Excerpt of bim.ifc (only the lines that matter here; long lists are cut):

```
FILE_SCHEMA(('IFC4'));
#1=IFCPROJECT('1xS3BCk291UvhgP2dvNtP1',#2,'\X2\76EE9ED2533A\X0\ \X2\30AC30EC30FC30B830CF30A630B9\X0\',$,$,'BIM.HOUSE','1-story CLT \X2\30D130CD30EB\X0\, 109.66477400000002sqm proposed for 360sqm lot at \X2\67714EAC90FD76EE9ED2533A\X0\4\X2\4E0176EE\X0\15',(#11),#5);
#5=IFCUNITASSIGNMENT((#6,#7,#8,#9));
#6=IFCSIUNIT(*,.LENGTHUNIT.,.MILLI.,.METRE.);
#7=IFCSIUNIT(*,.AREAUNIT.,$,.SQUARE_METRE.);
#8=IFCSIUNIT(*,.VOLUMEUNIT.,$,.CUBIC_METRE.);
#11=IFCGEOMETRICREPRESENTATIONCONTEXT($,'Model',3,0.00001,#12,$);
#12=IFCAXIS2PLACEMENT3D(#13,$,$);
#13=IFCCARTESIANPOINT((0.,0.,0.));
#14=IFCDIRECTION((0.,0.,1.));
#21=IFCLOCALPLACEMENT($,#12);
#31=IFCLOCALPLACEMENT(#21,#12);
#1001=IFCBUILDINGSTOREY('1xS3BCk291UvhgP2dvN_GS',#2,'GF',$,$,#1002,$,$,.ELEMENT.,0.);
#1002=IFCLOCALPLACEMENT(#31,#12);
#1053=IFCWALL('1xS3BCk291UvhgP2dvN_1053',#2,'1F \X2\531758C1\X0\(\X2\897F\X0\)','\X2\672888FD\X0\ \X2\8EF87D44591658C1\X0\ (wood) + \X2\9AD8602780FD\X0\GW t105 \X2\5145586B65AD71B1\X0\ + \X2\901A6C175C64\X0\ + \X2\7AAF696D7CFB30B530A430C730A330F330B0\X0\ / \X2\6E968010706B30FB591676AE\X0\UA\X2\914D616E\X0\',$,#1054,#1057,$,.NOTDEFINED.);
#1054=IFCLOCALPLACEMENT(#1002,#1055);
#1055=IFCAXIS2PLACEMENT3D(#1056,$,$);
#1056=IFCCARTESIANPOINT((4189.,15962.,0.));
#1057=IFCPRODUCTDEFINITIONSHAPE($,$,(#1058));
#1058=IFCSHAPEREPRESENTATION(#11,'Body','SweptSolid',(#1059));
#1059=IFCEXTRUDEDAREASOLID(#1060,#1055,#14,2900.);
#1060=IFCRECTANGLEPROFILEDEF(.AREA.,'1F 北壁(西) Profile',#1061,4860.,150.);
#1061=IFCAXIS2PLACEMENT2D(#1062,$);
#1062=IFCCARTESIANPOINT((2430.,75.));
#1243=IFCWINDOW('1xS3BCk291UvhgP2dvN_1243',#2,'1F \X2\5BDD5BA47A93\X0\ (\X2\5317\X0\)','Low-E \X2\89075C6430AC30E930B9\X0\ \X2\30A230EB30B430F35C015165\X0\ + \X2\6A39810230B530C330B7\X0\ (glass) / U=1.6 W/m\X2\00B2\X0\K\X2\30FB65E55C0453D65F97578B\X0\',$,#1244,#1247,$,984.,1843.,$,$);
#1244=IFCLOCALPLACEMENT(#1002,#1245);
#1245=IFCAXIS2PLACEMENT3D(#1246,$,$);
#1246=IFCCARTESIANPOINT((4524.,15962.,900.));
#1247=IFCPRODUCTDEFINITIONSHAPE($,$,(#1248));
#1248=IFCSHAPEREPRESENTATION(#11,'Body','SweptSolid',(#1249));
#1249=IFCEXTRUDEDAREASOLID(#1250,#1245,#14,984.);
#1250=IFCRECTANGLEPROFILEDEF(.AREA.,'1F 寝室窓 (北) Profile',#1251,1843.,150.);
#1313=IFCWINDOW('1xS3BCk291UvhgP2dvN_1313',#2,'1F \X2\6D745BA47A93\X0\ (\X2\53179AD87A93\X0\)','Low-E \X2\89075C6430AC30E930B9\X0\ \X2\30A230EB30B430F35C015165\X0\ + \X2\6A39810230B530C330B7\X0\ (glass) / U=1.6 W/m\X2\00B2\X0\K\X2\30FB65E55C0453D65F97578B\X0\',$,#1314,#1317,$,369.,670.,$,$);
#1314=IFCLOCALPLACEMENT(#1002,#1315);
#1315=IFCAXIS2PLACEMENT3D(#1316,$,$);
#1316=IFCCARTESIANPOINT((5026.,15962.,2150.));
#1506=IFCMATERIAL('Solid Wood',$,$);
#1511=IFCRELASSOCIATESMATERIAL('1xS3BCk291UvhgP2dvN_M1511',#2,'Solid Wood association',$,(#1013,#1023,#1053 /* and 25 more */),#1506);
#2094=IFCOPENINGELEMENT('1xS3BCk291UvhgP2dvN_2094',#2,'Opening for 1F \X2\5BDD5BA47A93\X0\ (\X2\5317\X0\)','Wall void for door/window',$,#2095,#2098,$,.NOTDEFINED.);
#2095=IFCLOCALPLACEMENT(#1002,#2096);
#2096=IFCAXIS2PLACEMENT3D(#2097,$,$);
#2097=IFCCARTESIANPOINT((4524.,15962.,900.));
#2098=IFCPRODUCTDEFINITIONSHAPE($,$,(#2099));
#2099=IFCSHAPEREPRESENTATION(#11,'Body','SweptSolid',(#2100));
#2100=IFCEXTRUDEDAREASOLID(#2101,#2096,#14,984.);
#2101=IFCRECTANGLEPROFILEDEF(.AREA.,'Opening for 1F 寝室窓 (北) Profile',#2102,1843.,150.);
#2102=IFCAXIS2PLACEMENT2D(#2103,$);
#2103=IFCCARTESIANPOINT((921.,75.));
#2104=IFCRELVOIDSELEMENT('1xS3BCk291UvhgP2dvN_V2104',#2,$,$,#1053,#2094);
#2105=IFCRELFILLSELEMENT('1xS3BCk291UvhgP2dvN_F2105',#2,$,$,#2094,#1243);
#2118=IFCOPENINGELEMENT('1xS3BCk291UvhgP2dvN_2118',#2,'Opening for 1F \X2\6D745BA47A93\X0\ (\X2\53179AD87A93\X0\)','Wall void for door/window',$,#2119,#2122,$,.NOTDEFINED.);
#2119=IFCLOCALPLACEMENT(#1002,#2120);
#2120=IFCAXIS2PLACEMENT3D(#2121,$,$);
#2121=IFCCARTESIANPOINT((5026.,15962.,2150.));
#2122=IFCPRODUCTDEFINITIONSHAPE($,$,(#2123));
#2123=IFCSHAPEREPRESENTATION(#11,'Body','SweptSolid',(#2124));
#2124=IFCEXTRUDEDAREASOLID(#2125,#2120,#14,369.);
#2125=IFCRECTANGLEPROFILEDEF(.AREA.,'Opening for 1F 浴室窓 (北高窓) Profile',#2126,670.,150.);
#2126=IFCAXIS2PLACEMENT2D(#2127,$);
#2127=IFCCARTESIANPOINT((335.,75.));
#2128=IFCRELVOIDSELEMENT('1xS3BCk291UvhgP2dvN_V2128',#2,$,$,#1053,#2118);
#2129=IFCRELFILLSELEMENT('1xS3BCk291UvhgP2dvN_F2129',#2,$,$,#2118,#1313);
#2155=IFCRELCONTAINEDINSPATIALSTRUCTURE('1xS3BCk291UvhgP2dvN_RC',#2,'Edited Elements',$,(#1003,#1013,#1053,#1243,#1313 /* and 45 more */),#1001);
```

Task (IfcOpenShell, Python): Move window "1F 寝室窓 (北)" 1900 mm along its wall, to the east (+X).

```python
import ifcopenshell
import ifcopenshell.api.geometry
import ifcopenshell.util.placement
import ifcopenshell.util.unit

model = ifcopenshell.open("bim.ifc")
unit_scale = ifcopenshell.util.unit.calculate_unit_scale(model)

window = model.by_guid("1xS3BCk291UvhgP2dvN_1243")
opening = window.FillsVoids[0].RelatingOpeningElement
wall = opening.VoidsElements[0].RelatingBuildingElement

wall_matrix = ifcopenshell.util.placement.get_local_placement(wall.ObjectPlacement)
shift = wall_matrix[:3, 0] * 1.9 / unit_scale
before = ifcopenshell.util.placement.get_local_placement(window.ObjectPlacement)[:3, 3].copy()

# The window is not placed relative to its opening, so move both.
for product in (opening, window):
    matrix = ifcopenshell.util.placement.get_local_placement(product.ObjectPlacement)
    matrix[:3, 3] += shift
    ifcopenshell.api.geometry.edit_object_placement(model, product=product, matrix=matrix, is_si=False)

after = ifcopenshell.util.placement.get_local_placement(window.ObjectPlacement)[:3, 3]
print("window moved by", (after - before).round(3) + 0.0)

model.write("bim_edited.ifc")
```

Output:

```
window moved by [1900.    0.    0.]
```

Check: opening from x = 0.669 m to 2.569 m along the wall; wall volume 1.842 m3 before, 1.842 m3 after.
